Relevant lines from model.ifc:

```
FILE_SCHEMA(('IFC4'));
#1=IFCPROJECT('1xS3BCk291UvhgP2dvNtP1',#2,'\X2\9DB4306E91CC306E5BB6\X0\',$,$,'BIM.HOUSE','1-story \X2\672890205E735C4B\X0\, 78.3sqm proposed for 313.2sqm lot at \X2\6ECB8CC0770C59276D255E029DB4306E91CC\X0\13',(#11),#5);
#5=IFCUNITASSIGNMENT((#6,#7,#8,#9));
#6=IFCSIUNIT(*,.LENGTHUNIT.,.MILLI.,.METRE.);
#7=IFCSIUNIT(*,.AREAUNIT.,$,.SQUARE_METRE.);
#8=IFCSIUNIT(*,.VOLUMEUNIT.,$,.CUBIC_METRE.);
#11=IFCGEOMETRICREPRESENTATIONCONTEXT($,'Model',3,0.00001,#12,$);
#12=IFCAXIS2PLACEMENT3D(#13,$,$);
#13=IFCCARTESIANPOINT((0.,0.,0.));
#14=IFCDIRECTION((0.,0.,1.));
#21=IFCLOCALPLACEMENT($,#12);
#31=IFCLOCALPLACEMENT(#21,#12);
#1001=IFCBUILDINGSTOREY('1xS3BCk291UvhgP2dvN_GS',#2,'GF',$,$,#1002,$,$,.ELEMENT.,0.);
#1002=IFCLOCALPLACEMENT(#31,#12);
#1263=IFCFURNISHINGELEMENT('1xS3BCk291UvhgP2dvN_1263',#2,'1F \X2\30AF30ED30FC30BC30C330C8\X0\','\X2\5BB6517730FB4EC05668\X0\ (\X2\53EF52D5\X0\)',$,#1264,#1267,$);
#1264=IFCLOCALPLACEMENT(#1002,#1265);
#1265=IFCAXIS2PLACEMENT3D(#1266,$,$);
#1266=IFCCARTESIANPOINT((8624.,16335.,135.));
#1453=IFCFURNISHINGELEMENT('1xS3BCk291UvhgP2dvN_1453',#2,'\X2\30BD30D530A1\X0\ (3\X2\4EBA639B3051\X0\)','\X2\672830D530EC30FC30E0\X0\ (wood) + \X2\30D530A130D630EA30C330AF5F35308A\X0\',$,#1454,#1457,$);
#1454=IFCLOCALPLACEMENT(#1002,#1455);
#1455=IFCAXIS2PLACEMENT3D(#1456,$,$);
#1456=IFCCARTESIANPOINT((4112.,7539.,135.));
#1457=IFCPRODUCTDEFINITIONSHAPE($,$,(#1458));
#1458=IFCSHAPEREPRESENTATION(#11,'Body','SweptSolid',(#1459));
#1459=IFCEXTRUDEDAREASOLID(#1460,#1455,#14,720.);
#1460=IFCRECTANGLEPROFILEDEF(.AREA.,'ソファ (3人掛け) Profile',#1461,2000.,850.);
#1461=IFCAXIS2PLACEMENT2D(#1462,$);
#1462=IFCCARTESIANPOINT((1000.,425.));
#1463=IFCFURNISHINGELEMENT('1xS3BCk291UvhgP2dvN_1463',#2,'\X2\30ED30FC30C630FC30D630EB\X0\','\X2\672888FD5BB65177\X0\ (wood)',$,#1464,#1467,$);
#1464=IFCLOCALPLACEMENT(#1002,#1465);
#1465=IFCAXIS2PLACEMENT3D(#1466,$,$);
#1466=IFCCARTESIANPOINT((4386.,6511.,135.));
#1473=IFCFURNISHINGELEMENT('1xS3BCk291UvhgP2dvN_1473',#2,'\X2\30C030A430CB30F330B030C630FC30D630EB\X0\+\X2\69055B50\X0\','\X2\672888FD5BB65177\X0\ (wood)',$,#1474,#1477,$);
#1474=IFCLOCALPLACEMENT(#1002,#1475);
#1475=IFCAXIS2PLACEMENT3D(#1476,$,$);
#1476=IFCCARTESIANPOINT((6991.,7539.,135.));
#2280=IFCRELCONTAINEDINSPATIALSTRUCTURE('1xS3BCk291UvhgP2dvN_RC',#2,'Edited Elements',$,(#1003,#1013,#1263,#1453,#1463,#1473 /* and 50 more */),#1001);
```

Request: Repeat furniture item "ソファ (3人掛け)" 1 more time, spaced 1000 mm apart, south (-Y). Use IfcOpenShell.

```python
import numpy as np
import ifcopenshell
import ifcopenshell.api.geometry
import ifcopenshell.api.root
import ifcopenshell.util.element
import ifcopenshell.util.placement

model = ifcopenshell.open("model.ifc")


def reuse_history(source, copy):
    """copy_class also copies each property set's owner history, people and application; keep the originals."""
    for rel in copy.IsDefinedBy:
        if rel.is_a("IfcRelDefinesByProperties") and (history := rel.RelatingPropertyDefinition.OwnerHistory):
            rel.RelatingPropertyDefinition.OwnerHistory = source.OwnerHistory
            ifcopenshell.util.element.remove_deep2(model, history)


source = model.by_guid("1xS3BCk291UvhgP2dvN_1453")
base = ifcopenshell.util.placement.get_local_placement(source.ObjectPlacement)
step = np.array([0.0, -1.0, 0.0]) * 1000.0

for i in range(1, 2):
    copy = ifcopenshell.api.root.copy_class(model, product=source)
    copy.Representation = ifcopenshell.util.element.copy_deep(
        model, source.Representation, exclude=["IfcGeometricRepresentationContext", "IfcRepresentationMap"]
    )
    reuse_history(source, copy)
    matrix = base.copy()
    matrix[:3, 3] += i * step
    print("added at", matrix[:3, 3].round(3) + 0.0)
    ifcopenshell.api.geometry.edit_object_placement(model, product=copy, matrix=matrix, is_si=False)

model.write("model_rev.ifc")
```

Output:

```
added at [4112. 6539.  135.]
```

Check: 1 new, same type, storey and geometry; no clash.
